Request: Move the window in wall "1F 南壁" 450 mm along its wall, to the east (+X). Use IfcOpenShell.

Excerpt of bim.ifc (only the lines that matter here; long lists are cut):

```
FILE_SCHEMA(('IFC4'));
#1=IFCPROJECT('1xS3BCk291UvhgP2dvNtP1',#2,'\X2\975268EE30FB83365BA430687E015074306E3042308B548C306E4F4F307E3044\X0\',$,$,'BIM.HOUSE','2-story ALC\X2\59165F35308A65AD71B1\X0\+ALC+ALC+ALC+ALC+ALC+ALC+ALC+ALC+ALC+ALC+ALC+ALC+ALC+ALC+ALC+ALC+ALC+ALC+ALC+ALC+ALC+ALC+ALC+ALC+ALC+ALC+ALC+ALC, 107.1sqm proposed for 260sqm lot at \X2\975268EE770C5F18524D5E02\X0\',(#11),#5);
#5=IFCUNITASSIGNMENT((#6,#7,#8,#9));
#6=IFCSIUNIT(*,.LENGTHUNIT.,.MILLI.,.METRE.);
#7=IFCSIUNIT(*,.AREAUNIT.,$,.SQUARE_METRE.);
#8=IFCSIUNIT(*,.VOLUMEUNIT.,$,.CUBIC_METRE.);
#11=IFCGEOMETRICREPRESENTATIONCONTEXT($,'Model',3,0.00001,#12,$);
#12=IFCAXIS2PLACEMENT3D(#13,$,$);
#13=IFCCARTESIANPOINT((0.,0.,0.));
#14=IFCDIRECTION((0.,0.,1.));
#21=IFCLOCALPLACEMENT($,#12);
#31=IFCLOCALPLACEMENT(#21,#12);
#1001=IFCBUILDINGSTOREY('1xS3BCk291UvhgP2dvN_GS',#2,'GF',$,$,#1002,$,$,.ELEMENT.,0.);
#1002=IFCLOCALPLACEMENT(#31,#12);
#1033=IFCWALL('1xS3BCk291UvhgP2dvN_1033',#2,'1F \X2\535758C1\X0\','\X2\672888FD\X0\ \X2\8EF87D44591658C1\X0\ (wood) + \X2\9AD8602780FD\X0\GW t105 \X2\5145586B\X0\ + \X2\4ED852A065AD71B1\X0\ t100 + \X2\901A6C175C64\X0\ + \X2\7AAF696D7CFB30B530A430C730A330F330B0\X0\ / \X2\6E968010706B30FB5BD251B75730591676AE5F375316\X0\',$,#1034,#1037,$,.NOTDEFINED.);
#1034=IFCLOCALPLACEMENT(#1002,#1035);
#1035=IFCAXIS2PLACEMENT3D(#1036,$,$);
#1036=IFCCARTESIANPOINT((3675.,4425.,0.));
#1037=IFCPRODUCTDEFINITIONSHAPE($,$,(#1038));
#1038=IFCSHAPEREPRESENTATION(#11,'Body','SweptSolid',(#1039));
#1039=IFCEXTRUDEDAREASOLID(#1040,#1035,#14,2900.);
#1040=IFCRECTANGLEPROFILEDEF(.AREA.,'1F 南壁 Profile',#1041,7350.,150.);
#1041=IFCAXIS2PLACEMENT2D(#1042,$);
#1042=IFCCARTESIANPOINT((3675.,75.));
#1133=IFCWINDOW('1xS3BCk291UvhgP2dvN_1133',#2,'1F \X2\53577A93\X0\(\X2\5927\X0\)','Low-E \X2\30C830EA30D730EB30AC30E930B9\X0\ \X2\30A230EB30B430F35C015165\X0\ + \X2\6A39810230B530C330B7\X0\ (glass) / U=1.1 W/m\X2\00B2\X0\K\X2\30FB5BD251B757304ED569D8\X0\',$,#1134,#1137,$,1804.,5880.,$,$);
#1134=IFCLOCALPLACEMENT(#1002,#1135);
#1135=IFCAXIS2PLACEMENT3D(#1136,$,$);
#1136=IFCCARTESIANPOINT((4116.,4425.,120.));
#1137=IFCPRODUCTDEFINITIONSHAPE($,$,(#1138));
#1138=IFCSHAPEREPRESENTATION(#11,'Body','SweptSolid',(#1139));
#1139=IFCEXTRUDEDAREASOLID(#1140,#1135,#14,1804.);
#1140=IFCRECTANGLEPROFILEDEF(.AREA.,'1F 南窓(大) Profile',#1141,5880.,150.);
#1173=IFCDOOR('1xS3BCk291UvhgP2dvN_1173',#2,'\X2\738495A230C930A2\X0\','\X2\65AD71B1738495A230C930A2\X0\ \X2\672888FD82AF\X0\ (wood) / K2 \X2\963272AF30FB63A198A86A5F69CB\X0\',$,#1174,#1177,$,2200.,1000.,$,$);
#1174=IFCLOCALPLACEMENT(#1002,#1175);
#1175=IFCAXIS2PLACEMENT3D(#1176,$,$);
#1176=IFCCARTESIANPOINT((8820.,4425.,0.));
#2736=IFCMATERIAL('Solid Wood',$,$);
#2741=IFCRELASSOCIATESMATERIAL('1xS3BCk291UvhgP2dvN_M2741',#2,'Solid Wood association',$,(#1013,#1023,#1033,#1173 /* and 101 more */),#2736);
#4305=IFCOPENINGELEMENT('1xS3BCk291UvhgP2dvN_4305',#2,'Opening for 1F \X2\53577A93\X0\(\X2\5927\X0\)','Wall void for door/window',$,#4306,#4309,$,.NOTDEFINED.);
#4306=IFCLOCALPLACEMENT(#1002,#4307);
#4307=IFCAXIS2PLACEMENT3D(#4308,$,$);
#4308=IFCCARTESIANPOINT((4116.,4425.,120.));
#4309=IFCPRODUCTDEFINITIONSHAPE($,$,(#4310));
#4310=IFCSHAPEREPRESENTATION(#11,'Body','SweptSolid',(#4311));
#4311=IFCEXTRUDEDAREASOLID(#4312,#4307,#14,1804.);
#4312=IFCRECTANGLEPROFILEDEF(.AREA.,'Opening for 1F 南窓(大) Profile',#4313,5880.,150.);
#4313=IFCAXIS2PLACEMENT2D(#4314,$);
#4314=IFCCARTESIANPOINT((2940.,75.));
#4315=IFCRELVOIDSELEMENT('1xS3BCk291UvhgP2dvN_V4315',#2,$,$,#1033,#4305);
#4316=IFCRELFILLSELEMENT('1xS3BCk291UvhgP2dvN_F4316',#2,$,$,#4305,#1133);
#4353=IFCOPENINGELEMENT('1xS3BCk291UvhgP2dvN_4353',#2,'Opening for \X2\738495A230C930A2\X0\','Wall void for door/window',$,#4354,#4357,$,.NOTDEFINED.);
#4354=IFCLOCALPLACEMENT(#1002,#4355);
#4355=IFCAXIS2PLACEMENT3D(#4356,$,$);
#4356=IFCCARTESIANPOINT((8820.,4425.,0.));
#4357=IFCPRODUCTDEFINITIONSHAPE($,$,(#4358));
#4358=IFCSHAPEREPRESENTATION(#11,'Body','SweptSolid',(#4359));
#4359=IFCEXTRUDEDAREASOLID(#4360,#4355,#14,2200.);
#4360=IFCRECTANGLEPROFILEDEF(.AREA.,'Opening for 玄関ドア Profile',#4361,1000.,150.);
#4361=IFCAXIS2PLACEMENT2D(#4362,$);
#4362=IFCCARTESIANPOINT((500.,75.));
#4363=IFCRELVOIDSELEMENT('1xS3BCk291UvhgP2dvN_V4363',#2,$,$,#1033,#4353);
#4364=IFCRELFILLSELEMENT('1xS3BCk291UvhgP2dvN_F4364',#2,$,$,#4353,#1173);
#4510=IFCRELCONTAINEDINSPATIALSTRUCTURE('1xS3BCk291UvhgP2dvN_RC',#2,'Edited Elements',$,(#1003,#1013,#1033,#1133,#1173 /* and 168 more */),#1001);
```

```python
import ifcopenshell
import ifcopenshell.api.geometry
import ifcopenshell.util.placement
import ifcopenshell.util.unit

model = ifcopenshell.open("bim.ifc")
unit_scale = ifcopenshell.util.unit.calculate_unit_scale(model)

window = model.by_guid("1xS3BCk291UvhgP2dvN_1133")
opening = window.FillsVoids[0].RelatingOpeningElement
wall = opening.VoidsElements[0].RelatingBuildingElement

wall_matrix = ifcopenshell.util.placement.get_local_placement(wall.ObjectPlacement)
shift = wall_matrix[:3, 0] * 0.45 / unit_scale
before = ifcopenshell.util.placement.get_local_placement(window.ObjectPlacement)[:3, 3].copy()

# The window is not placed relative to its opening, so move both.
for product in (opening, window):
    matrix = ifcopenshell.util.placement.get_local_placement(product.ObjectPlacement)
    matrix[:3, 3] += shift
    ifcopenshell.api.geometry.edit_object_placement(model, product=product, matrix=matrix, is_si=False)

after = ifcopenshell.util.placement.get_local_placement(window.ObjectPlacement)[:3, 3]
print("window moved by", (after - before).round(3) + 0.0)

model.write("bim_v2.ifc")
```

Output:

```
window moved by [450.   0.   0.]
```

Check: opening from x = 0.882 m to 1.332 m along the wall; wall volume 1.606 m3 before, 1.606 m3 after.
